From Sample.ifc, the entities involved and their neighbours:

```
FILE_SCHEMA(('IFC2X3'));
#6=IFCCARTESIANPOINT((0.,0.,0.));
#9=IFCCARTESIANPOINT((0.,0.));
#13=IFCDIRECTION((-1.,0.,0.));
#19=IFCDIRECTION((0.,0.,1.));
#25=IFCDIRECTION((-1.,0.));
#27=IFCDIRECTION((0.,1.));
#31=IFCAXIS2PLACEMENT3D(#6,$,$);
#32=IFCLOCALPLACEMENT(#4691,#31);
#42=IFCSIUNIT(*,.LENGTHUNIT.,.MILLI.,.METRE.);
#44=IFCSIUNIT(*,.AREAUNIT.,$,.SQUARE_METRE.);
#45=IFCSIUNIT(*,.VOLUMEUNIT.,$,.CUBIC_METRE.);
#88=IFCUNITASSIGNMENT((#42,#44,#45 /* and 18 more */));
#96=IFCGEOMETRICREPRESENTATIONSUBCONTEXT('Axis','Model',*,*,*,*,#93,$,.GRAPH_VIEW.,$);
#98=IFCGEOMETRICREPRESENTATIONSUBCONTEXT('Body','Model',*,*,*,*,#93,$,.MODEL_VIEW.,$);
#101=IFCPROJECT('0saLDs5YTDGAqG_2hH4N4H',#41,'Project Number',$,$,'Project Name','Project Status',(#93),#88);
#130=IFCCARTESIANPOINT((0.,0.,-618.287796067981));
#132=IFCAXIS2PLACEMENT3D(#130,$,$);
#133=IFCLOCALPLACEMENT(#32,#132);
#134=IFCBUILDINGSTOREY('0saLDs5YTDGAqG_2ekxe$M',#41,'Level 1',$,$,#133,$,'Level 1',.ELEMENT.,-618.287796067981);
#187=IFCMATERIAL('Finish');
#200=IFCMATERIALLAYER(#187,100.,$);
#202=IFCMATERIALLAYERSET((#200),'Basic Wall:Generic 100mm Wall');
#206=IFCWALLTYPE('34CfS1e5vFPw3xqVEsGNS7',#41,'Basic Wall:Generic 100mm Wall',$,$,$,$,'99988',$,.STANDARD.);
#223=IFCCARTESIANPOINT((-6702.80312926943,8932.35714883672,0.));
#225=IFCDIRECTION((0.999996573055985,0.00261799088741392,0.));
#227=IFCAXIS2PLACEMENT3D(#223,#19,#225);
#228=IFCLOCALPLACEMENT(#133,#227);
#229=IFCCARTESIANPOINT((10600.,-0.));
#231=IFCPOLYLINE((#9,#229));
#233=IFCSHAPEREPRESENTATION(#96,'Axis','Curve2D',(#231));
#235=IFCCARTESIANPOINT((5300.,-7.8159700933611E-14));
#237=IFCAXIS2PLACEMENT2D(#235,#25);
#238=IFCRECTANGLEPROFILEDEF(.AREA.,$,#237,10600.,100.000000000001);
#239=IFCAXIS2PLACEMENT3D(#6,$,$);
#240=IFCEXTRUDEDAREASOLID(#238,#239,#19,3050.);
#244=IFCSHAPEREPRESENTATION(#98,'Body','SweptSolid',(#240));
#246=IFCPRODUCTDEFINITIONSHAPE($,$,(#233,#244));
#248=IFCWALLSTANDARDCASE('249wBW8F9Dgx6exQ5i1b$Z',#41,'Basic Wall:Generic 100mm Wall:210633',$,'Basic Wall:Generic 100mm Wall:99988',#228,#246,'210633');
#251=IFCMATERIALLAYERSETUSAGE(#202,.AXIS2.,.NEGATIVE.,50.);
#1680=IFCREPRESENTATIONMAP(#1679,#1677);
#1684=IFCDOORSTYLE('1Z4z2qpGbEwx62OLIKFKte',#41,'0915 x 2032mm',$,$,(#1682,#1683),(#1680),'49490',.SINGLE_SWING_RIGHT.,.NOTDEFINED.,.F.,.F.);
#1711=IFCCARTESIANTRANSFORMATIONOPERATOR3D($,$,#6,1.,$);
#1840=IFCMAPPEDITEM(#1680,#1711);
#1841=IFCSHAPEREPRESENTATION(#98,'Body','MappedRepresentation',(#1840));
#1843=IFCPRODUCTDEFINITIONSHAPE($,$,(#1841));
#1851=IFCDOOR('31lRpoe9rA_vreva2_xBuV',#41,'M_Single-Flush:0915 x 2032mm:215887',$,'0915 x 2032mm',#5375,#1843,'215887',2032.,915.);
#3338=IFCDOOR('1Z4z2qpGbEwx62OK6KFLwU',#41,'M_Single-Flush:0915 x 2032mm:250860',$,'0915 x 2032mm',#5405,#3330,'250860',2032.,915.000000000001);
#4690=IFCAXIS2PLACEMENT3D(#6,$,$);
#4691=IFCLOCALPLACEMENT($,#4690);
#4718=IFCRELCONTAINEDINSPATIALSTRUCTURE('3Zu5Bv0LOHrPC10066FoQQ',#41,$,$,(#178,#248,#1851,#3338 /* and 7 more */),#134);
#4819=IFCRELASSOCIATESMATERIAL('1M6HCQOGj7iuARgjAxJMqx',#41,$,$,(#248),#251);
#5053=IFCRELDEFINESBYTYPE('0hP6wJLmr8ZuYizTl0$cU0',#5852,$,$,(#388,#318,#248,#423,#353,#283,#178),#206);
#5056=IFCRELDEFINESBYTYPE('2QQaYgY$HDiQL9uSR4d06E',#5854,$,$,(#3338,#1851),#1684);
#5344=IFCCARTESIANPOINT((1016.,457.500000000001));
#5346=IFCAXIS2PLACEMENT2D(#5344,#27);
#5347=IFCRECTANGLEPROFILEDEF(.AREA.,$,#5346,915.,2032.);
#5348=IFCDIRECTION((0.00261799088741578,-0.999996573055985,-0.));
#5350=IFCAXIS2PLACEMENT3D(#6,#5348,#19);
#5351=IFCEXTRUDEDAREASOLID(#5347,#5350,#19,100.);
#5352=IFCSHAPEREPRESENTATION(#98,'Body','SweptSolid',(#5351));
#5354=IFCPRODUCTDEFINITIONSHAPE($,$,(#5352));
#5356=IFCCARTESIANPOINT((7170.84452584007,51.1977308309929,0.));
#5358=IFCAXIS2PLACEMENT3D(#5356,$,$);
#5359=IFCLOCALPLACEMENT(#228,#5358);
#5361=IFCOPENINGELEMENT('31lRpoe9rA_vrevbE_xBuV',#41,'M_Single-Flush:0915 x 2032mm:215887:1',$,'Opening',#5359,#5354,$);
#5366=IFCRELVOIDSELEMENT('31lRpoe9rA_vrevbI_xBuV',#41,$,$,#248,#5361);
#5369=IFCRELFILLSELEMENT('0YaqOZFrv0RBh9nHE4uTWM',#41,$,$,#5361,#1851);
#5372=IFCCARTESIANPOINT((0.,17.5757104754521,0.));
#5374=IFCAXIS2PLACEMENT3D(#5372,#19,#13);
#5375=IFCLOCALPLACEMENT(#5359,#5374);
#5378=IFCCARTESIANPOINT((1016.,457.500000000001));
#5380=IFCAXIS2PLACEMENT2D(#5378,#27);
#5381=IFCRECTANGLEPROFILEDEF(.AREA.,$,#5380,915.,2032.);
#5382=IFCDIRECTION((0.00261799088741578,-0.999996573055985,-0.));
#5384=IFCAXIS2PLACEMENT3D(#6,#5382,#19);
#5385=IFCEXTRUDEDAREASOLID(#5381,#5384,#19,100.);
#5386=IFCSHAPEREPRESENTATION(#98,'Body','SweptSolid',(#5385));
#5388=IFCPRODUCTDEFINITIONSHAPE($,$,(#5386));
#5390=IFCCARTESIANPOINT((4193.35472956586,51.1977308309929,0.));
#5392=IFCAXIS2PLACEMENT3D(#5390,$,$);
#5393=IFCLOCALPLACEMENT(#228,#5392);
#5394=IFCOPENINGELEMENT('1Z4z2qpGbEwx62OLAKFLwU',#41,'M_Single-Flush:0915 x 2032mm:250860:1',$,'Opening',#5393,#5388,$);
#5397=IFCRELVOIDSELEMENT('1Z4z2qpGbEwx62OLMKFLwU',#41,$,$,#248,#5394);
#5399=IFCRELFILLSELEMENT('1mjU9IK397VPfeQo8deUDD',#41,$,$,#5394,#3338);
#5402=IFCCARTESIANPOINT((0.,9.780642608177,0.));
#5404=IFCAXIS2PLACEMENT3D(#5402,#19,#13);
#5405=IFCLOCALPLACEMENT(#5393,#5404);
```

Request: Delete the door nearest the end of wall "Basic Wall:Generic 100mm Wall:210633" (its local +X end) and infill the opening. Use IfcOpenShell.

```python
import ifcopenshell
import ifcopenshell.api.feature
import ifcopenshell.api.root
import ifcopenshell.geom
import ifcopenshell.util.shape

model = ifcopenshell.open("Sample.ifc")
settings = ifcopenshell.geom.settings()


def volume(element):
    """Net volume in cubic metres, openings subtracted."""
    shape = ifcopenshell.geom.create_shape(settings, element)
    return ifcopenshell.util.shape.get_volume(shape.geometry)


door = model.by_guid("31lRpoe9rA_vreva2_xBuV")
opening = door.FillsVoids[0].RelatingOpeningElement
wall = opening.VoidsElements[0].RelatingBuildingElement
before = volume(wall)

ifcopenshell.api.root.remove_product(model, product=door)
ifcopenshell.api.feature.remove_feature(model, feature=opening)

after = volume(wall)

print(f"wall volume {before:.3f} -> {after:.3f} m3")

model.write("Sample_updated.ifc")
```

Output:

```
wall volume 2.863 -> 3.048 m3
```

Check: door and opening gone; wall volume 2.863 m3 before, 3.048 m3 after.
